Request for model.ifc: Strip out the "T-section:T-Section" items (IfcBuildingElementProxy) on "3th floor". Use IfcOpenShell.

First a look at what the model holds.

```python
import ifcopenshell
import ifcopenshell.util.element

model = ifcopenshell.open("model.ifc")
print(model.schema)
storey = next(s for s in model.by_type("IfcBuildingStorey") if s.Name == "3th floor")
proxies = [e for e in ifcopenshell.util.element.get_decomposition(storey) if e.is_a("IfcBuildingElementProxy")]
seen = {}
for e in proxies:
    element_type = ifcopenshell.util.element.get_type(e)
    name = element_type.Name if element_type not in (None, e) else None
    seen[name] = seen.get(name, 0) + 1
for name, count in sorted(seen.items(), key=str):
    print(count, "x", name)
```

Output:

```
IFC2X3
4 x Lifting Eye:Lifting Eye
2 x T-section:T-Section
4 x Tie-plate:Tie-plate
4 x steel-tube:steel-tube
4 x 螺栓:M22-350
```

```python
import ifcopenshell
import ifcopenshell.api.root
import ifcopenshell.util.element

model = ifcopenshell.open("model.ifc")

storey = next(s for s in model.by_type("IfcBuildingStorey") if s.Name == "3th floor")
proxies = [e for e in ifcopenshell.util.element.get_decomposition(storey) if e.is_a("IfcBuildingElementProxy")]
targets = [e for e in proxies if (t := ifcopenshell.util.element.get_type(e)) not in (None, e) and t.Name == "T-section:T-Section"]

for e in targets:
    ifcopenshell.api.root.remove_product(model, product=e)
print(len(targets), "removed")

model.write("model-out.ifc")
```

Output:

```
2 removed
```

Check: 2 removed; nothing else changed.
